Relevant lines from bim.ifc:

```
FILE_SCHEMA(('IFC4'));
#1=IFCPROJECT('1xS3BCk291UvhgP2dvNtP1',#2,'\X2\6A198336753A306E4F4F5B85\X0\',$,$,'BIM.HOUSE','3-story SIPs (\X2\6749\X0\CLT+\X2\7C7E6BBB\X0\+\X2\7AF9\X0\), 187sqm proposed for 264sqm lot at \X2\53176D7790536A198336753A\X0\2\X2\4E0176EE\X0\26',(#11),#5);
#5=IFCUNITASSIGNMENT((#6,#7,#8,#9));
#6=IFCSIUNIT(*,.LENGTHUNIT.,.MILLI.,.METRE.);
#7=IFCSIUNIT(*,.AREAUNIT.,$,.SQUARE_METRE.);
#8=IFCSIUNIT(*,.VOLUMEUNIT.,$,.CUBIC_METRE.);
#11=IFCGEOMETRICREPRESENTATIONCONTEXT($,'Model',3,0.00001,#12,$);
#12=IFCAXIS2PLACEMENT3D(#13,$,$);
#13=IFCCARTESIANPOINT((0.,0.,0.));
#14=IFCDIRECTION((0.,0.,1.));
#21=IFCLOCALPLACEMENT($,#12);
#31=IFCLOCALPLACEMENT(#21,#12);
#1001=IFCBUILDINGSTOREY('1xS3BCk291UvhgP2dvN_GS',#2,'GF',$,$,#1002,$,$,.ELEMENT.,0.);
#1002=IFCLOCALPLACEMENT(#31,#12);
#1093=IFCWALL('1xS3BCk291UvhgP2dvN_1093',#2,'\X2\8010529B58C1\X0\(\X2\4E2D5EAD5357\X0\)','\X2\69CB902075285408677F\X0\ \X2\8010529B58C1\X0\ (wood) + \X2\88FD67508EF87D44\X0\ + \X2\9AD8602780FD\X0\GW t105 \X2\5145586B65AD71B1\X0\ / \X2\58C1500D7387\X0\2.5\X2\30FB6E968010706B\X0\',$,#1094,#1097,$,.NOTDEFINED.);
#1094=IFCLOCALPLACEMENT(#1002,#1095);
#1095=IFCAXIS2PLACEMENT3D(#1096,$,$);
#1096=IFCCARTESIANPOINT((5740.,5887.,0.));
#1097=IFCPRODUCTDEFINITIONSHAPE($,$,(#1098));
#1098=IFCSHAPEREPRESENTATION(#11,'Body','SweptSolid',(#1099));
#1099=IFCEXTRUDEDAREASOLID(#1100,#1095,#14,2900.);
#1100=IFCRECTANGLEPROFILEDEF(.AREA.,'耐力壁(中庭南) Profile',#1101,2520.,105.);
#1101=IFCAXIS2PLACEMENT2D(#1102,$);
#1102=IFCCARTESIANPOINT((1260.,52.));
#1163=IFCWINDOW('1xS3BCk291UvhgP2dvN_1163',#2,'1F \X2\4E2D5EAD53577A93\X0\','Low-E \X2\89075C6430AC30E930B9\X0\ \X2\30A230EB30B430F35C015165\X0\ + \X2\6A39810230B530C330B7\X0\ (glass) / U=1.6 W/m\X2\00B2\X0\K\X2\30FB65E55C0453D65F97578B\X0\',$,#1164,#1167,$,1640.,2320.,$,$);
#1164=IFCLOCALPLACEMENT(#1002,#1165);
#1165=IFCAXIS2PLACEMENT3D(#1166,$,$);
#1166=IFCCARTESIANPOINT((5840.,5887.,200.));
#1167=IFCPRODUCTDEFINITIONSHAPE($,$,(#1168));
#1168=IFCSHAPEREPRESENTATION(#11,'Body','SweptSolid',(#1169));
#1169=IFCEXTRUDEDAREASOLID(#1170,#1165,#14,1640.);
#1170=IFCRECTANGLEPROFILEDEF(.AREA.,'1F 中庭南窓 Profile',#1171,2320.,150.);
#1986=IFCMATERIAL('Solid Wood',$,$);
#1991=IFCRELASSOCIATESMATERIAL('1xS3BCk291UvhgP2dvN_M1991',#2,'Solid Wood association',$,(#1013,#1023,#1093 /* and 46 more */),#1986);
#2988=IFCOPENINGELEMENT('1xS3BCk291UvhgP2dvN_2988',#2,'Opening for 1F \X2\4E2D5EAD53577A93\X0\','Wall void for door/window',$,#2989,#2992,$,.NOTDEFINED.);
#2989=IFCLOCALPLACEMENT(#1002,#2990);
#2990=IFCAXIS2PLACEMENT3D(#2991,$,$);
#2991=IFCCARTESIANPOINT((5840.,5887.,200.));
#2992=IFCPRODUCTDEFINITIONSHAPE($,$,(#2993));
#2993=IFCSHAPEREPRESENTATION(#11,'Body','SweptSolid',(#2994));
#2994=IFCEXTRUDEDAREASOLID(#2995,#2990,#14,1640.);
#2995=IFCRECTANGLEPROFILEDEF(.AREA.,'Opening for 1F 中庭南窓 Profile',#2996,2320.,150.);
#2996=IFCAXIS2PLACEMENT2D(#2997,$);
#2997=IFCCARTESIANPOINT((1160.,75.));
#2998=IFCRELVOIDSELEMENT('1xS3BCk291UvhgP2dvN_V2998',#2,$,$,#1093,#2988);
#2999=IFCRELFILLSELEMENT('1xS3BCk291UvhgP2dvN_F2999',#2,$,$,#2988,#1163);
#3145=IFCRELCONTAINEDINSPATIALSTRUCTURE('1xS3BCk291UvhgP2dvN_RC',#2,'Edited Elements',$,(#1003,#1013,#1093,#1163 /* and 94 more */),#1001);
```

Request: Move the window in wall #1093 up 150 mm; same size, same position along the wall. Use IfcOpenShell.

```python
import numpy as np
import ifcopenshell
import ifcopenshell.api.geometry
import ifcopenshell.util.placement
import ifcopenshell.util.unit

model = ifcopenshell.open("bim.ifc")
unit_scale = ifcopenshell.util.unit.calculate_unit_scale(model)

window = model.by_id(1163)
opening = window.FillsVoids[0].RelatingOpeningElement
dz = 150.0

shift = np.array([0.0, 0.0, dz])
# The window is not placed relative to its opening, so move both.
for product in (opening, window):
    matrix = ifcopenshell.util.placement.get_local_placement(product.ObjectPlacement)
    matrix[:3, 3] += shift
    ifcopenshell.api.geometry.edit_object_placement(model, product=product, matrix=matrix, is_si=False)

print(f"moved by {dz * unit_scale:+.3f} m")

model.write("bim-out.ifc")
```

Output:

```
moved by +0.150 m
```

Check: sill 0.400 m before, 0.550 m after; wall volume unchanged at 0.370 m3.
